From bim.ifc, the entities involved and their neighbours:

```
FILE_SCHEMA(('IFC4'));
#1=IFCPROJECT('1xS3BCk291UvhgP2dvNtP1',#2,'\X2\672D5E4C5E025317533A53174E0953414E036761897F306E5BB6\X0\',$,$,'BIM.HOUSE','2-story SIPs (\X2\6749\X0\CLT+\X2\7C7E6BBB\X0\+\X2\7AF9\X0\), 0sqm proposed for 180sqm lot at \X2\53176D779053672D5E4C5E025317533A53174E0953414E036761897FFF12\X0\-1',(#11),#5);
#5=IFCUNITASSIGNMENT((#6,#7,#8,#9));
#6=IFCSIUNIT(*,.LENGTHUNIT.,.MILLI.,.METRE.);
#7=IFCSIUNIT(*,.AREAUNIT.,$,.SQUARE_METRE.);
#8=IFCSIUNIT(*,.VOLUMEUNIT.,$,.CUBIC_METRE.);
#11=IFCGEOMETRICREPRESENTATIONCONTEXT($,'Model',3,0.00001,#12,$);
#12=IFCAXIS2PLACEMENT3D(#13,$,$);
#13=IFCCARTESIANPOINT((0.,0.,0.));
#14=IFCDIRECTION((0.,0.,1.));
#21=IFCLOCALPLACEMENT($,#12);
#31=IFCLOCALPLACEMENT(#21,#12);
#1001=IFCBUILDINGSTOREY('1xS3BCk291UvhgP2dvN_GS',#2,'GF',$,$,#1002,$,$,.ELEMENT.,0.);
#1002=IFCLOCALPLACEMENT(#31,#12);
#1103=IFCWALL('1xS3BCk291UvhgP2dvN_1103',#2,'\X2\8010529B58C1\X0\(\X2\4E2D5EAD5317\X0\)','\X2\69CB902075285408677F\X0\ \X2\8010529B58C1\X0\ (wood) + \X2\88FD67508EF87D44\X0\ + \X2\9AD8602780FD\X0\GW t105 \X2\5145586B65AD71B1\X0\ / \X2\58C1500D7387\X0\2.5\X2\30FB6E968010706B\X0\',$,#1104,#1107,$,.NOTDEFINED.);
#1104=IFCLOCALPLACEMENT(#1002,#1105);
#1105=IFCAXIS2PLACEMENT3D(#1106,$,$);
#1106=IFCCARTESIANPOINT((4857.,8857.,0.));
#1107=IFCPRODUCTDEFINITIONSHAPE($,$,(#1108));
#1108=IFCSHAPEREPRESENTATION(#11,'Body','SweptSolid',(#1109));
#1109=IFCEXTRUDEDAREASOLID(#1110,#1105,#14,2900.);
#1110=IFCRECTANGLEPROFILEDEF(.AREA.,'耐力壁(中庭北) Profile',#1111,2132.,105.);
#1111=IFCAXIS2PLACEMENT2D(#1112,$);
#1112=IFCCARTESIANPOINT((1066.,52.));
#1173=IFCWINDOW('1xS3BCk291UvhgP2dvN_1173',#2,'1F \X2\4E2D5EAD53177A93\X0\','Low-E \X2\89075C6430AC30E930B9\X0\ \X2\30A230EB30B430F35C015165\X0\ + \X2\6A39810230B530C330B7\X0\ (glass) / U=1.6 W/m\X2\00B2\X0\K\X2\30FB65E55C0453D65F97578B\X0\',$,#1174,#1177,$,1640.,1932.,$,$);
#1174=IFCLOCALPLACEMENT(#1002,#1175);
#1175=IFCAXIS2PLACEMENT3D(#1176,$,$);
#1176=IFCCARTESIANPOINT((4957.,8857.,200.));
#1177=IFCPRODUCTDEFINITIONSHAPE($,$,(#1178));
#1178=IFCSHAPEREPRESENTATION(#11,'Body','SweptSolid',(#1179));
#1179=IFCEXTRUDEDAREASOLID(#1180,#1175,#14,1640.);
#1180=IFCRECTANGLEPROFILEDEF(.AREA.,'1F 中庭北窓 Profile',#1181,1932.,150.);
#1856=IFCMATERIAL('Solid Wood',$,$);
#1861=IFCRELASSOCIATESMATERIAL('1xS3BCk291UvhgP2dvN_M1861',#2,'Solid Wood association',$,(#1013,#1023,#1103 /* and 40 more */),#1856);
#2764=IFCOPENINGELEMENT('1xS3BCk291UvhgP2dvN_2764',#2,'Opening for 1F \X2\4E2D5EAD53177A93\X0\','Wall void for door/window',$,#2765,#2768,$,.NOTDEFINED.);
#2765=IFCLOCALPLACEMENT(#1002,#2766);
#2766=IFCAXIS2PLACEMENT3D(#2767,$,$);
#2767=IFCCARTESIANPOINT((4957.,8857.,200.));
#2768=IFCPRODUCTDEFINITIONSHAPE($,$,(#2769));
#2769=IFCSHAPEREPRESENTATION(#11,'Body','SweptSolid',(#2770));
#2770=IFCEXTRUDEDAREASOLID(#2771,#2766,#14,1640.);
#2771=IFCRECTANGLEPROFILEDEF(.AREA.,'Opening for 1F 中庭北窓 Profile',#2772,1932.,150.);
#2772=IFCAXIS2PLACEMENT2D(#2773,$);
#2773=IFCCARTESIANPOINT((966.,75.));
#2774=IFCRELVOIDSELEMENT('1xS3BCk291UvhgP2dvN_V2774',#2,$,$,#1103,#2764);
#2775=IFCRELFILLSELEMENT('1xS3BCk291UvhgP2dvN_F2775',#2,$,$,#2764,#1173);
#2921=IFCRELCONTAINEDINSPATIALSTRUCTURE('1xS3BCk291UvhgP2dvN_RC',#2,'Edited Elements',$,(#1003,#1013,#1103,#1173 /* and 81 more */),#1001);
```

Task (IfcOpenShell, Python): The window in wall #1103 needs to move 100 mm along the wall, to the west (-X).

```python
import ifcopenshell
import ifcopenshell.api.geometry
import ifcopenshell.util.placement
import ifcopenshell.util.unit

model = ifcopenshell.open("bim.ifc")
unit_scale = ifcopenshell.util.unit.calculate_unit_scale(model)

window = model.by_guid("1xS3BCk291UvhgP2dvN_1173")
opening = window.FillsVoids[0].RelatingOpeningElement
wall = opening.VoidsElements[0].RelatingBuildingElement

wall_matrix = ifcopenshell.util.placement.get_local_placement(wall.ObjectPlacement)
shift = wall_matrix[:3, 0] * -0.1 / unit_scale
before = ifcopenshell.util.placement.get_local_placement(window.ObjectPlacement)[:3, 3].copy()

# The window is not placed relative to its opening, so move both.
for product in (opening, window):
    matrix = ifcopenshell.util.placement.get_local_placement(product.ObjectPlacement)
    matrix[:3, 3] += shift
    ifcopenshell.api.geometry.edit_object_placement(model, product=product, matrix=matrix, is_si=False)

after = ifcopenshell.util.placement.get_local_placement(window.ObjectPlacement)[:3, 3]
print("window moved by", (after - before).round(3) + 0.0)

model.write("bim_edited.ifc")
```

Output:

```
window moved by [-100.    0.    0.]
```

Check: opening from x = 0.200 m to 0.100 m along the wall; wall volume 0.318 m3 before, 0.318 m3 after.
